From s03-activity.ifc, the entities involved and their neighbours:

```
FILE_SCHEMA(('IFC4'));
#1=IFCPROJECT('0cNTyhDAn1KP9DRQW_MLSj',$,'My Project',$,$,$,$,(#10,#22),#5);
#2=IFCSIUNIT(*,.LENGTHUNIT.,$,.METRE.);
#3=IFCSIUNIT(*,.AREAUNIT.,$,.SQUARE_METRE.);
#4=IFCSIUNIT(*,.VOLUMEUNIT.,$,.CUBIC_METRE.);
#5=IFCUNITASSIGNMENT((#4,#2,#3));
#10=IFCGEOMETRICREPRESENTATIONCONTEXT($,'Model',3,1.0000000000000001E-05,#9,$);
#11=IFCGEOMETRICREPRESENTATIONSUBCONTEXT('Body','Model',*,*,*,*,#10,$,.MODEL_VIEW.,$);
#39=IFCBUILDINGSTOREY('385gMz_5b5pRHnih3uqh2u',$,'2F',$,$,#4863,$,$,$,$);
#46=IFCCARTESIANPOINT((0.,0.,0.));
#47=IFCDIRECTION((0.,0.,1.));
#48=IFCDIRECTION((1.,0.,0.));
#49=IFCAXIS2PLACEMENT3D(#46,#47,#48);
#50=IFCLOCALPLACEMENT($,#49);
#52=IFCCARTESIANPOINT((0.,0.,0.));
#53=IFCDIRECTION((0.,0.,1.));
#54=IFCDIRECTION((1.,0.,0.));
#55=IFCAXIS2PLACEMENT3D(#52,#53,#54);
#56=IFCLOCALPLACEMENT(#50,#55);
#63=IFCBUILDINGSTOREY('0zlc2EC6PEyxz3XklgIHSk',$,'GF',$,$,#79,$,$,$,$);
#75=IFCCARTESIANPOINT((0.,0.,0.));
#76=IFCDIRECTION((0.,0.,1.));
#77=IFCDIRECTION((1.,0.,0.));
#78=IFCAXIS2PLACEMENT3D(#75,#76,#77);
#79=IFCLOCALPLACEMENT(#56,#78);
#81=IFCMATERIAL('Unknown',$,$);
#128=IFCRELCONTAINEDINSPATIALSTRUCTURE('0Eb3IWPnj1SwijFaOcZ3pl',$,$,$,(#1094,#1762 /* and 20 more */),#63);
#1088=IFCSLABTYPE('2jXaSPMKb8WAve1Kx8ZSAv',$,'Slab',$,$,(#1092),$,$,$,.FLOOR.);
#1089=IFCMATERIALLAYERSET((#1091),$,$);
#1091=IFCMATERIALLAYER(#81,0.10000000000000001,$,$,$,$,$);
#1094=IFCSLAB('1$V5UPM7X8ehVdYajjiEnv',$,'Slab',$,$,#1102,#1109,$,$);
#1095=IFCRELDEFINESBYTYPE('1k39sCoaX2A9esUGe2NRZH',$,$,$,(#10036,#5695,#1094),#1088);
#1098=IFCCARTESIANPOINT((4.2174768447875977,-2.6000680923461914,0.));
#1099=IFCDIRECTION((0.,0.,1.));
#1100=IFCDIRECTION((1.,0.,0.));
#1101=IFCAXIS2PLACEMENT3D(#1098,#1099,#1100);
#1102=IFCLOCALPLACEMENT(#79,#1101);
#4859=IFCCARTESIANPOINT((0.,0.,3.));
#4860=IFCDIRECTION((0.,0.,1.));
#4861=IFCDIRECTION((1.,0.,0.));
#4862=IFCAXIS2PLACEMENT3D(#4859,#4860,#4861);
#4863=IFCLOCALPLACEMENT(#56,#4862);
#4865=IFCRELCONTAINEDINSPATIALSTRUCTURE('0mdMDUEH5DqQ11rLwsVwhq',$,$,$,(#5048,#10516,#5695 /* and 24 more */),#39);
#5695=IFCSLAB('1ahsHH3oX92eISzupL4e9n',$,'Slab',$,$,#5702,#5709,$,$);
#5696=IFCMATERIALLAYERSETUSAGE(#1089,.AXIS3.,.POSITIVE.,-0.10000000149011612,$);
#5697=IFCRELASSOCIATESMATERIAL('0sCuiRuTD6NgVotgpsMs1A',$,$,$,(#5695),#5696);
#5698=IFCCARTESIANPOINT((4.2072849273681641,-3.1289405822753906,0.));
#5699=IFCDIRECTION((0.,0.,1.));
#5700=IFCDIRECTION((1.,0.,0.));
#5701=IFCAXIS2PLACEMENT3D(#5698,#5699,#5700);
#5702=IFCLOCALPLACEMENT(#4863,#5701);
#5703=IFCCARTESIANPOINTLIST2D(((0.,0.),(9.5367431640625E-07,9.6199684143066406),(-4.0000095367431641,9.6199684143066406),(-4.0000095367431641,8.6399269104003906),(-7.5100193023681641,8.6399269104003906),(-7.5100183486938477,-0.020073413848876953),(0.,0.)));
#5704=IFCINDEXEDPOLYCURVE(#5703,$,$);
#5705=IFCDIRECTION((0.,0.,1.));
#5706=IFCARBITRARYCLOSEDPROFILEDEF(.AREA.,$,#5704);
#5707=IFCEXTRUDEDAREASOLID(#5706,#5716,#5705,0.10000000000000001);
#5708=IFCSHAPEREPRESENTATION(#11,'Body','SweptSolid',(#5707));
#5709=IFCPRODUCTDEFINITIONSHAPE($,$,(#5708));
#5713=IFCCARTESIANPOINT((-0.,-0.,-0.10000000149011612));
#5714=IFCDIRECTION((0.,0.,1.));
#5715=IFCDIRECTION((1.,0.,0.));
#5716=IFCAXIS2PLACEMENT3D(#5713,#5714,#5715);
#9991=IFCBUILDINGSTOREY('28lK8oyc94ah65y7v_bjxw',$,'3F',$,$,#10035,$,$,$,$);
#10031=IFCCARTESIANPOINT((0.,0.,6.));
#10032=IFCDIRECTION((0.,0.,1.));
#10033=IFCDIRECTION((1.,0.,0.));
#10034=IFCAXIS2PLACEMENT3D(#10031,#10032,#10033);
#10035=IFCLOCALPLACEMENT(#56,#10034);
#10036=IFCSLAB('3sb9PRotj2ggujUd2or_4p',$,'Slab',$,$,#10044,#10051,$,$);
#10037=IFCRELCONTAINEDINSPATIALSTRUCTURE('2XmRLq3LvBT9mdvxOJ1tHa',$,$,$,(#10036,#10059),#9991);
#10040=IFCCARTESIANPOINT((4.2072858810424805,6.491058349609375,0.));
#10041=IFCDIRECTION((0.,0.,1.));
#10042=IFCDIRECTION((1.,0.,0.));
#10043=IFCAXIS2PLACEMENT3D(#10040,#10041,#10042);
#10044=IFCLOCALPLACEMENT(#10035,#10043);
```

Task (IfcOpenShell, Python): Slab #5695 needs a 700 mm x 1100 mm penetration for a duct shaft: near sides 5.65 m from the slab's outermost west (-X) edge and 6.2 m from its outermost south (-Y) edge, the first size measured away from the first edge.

```python
import numpy as np
import ifcopenshell
import ifcopenshell.api.feature
import ifcopenshell.api.geometry
import ifcopenshell.api.root
import ifcopenshell.geom
import ifcopenshell.util.placement
import ifcopenshell.util.representation
import ifcopenshell.util.shape
import ifcopenshell.util.unit

model = ifcopenshell.open("s03-activity.ifc")
unit_scale = ifcopenshell.util.unit.calculate_unit_scale(model)
settings = ifcopenshell.geom.settings()


def volume(element):
    """Net volume in cubic metres, openings subtracted."""
    shape = ifcopenshell.geom.create_shape(settings, element)
    return ifcopenshell.util.shape.get_volume(shape.geometry)


slab = model.by_guid("1ahsHH3oX92eISzupL4e9n")
before = volume(slab)

# Extent in the slab's own axes, in metres. The edges named are its -X and -Y sides.
slab_shape = ifcopenshell.geom.create_shape(settings, slab)
vertices = ifcopenshell.util.shape.get_vertices(slab_shape.geometry)
x_min, y_min, bottom = vertices.min(axis=0)
top = vertices[:, 2].max()

opening = ifcopenshell.api.root.create_entity(model, ifc_class="IfcOpeningElement", name="Duct shaft opening", predefined_type="OPENING")
context = ifcopenshell.util.representation.get_context(model, "Model", "Body", "MODEL_VIEW")
width, depth = 0.7, 1.1
outline = [(0.0, 0.0), (width, 0.0), (width, depth), (0.0, depth), (0.0, 0.0)]
# Overshoot both faces by 50 mm so the cut is clean.
shape = ifcopenshell.api.geometry.add_slab_representation(
    model, context=context, depth=top - bottom + 0.1, polyline=outline
)
ifcopenshell.api.geometry.assign_representation(model, product=opening, representation=shape)

matrix = ifcopenshell.util.placement.get_local_placement(slab.ObjectPlacement)
matrix[:, 3] = matrix @ np.append(np.array([x_min + 5.65, y_min + 6.2, bottom - 0.05]) / unit_scale, 1.0)
ifcopenshell.api.geometry.edit_object_placement(model, product=opening, matrix=matrix, is_si=False)
ifcopenshell.api.feature.add_feature(model, feature=opening, element=slab)

after = volume(slab)

print(f"slab volume {before:.3f} -> {after:.3f} m3")

model.write("s03-activity_rev.ifc")
```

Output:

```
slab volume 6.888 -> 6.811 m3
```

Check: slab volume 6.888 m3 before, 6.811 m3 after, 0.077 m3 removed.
